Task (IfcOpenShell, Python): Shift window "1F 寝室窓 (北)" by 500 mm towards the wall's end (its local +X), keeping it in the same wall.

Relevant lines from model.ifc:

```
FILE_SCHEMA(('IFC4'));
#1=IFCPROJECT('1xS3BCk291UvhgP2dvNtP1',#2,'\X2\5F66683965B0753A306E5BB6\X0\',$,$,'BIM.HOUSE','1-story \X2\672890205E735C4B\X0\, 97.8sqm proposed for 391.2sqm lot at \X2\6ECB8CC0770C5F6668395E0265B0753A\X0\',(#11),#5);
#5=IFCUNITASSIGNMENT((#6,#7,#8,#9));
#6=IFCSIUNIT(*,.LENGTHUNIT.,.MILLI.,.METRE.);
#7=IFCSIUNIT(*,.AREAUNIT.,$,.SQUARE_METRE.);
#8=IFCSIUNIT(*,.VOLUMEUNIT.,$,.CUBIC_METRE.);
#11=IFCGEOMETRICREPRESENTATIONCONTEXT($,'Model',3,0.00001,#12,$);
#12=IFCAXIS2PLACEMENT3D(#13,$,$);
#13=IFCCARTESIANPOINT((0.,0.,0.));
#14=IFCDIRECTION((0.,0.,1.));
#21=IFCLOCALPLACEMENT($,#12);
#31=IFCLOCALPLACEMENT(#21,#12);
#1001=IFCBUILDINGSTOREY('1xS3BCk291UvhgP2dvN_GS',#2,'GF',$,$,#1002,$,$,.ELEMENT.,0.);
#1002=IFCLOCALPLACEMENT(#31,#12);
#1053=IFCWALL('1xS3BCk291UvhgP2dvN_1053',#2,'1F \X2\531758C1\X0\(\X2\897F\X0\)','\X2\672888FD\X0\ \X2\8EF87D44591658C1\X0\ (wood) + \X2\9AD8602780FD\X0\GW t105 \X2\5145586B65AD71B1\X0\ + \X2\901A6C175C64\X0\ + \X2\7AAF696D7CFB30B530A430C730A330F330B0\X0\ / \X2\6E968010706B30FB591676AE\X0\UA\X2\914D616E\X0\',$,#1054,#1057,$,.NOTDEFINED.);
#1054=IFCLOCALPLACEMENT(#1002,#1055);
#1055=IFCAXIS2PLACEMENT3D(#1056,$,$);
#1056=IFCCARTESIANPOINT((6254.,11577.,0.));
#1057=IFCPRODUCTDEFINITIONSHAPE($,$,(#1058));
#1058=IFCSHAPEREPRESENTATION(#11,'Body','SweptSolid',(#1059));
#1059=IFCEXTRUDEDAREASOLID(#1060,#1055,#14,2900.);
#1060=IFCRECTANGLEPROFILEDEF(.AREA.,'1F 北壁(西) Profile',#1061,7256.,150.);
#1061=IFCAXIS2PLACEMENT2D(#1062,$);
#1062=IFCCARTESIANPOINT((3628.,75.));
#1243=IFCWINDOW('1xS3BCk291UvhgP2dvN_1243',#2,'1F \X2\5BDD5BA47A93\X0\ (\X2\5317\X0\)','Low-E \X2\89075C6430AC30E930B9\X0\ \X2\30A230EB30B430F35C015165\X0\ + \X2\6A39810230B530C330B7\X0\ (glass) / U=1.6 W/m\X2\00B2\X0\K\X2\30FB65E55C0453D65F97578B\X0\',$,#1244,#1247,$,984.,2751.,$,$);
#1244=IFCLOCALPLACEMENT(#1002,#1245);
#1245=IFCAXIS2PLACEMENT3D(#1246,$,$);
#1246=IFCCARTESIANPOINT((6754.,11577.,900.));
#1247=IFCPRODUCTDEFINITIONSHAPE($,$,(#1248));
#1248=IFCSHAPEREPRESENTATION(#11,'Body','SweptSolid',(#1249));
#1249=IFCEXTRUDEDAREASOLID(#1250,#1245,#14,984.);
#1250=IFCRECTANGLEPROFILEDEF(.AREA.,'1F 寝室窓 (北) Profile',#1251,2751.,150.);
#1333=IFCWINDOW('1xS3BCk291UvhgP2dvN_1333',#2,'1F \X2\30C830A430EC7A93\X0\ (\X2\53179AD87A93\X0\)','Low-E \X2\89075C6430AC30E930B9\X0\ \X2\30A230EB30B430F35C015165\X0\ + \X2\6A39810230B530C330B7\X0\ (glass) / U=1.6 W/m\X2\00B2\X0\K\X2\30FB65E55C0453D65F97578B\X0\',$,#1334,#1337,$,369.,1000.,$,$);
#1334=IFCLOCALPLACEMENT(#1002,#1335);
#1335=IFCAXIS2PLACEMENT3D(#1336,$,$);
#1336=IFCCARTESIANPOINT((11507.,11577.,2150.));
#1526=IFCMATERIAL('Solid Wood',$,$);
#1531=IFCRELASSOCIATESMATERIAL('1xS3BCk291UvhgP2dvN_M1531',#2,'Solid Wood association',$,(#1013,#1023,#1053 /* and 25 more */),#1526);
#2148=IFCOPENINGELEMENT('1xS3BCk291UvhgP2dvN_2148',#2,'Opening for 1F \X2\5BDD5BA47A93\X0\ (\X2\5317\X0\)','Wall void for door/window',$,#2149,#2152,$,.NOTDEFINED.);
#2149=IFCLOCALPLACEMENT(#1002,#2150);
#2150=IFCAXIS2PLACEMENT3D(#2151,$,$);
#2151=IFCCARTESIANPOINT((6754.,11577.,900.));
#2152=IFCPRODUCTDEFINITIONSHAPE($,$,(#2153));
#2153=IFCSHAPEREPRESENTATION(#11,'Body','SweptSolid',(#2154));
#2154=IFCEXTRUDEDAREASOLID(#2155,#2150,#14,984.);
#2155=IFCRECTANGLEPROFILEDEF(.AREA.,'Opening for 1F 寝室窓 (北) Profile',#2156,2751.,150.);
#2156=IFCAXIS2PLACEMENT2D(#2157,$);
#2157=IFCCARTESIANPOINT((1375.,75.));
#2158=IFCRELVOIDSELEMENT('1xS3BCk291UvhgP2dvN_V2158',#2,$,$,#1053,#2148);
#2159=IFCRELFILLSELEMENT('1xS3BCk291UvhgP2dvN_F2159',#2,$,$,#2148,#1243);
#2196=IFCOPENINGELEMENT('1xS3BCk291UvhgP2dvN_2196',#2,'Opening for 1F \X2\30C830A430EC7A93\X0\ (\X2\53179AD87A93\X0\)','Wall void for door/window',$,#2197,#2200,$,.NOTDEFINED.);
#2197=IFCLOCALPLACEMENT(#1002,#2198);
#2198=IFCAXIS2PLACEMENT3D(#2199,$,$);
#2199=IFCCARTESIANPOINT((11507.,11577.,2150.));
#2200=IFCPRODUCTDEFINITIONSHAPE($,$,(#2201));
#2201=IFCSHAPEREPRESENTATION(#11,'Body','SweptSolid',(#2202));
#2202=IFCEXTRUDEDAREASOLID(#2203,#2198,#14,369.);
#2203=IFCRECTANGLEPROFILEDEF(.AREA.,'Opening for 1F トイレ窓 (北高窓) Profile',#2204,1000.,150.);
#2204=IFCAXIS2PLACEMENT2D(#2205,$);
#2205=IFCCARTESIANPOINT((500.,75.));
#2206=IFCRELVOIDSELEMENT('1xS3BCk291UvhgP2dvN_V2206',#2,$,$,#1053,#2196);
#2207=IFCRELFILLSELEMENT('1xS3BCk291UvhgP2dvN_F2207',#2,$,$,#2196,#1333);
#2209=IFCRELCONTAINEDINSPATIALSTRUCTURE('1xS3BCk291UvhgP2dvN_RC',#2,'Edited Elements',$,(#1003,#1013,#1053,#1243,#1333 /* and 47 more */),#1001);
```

```python
import ifcopenshell
import ifcopenshell.api.geometry
import ifcopenshell.util.placement
import ifcopenshell.util.unit

model = ifcopenshell.open("model.ifc")
unit_scale = ifcopenshell.util.unit.calculate_unit_scale(model)

window = model.by_guid("1xS3BCk291UvhgP2dvN_1243")
opening = window.FillsVoids[0].RelatingOpeningElement
wall = opening.VoidsElements[0].RelatingBuildingElement

wall_matrix = ifcopenshell.util.placement.get_local_placement(wall.ObjectPlacement)
shift = wall_matrix[:3, 0] * 0.5 / unit_scale
before = ifcopenshell.util.placement.get_local_placement(window.ObjectPlacement)[:3, 3].copy()

# The window is not placed relative to its opening, so move both.
for product in (opening, window):
    matrix = ifcopenshell.util.placement.get_local_placement(product.ObjectPlacement)
    matrix[:3, 3] += shift
    ifcopenshell.api.geometry.edit_object_placement(model, product=product, matrix=matrix, is_si=False)

after = ifcopenshell.util.placement.get_local_placement(window.ObjectPlacement)[:3, 3]
print("window moved by", (after - before).round(3) + 0.0)

model.write("model-out.ifc")
```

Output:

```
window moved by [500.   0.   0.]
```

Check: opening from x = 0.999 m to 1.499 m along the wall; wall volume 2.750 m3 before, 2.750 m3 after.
